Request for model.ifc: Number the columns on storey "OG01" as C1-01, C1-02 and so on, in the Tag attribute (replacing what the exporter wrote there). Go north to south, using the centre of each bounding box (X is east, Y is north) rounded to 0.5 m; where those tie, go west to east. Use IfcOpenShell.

First a look at what the model holds.

```python
import ifcopenshell
import ifcopenshell.util.element
import ifcopenshell.util.placement

model = ifcopenshell.open("model.ifc")
print(model.schema)
storey = next(s for s in model.by_type("IfcBuildingStorey") if s.Name == "OG01")
columns = [e for e in ifcopenshell.util.element.get_decomposition(storey) if e.is_a("IfcColumn")]
for e in sorted(columns, key=lambda e: e.id()):
    origin = ifcopenshell.util.placement.get_local_placement(e.ObjectPlacement)[:3, 3]
    print(e.id(), e.Tag, e.Name, origin.round(2) + 0.0, sep=" | ")
```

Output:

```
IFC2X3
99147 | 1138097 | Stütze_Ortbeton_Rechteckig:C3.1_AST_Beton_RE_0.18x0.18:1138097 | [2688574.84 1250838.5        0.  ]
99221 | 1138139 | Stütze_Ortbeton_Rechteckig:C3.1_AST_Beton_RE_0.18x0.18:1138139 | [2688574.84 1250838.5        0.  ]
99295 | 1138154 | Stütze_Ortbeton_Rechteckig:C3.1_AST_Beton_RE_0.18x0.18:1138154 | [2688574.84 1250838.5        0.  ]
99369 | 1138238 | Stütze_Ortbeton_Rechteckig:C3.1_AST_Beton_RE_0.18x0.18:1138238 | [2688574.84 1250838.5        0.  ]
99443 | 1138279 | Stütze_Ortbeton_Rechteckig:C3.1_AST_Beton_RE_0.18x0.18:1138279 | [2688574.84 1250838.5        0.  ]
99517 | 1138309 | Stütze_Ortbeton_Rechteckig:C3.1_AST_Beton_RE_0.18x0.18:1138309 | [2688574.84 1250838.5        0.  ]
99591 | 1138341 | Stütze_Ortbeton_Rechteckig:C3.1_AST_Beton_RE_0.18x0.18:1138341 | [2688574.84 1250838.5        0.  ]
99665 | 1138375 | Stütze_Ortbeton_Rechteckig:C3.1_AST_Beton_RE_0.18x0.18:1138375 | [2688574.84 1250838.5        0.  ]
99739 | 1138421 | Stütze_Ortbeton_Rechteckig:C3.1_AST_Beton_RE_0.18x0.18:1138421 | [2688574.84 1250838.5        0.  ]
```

```python
import ifcopenshell
import ifcopenshell.geom
import ifcopenshell.util.element
import ifcopenshell.util.shape

model = ifcopenshell.open("model.ifc")
settings = ifcopenshell.geom.settings()
settings.set("use-world-coords", True)


def centre(element):
    shape = ifcopenshell.geom.create_shape(settings, element)
    return ifcopenshell.util.shape.get_bbox_centroid(shape.geometry)


storey = next(s for s in model.by_type("IfcBuildingStorey") if s.Name == "OG01")
columns = [e for e in ifcopenshell.util.element.get_decomposition(storey) if e.is_a("IfcColumn")]

# Insertion points can sit at a corner or the storey origin, so sort by the geometry (in metres).
centres = {e: centre(e) for e in columns}
columns.sort(key=lambda e: (-round(centres[e][1] / 0.5), centres[e][0]))

for i, e in enumerate(columns, start=1):
    number = f"C1-{i:02d}"
    e.Tag = number
    print(e.id(), number)

model.write("model_edited.ifc")
```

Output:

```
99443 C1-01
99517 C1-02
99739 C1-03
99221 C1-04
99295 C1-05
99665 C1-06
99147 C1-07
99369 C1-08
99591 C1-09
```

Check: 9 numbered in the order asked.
